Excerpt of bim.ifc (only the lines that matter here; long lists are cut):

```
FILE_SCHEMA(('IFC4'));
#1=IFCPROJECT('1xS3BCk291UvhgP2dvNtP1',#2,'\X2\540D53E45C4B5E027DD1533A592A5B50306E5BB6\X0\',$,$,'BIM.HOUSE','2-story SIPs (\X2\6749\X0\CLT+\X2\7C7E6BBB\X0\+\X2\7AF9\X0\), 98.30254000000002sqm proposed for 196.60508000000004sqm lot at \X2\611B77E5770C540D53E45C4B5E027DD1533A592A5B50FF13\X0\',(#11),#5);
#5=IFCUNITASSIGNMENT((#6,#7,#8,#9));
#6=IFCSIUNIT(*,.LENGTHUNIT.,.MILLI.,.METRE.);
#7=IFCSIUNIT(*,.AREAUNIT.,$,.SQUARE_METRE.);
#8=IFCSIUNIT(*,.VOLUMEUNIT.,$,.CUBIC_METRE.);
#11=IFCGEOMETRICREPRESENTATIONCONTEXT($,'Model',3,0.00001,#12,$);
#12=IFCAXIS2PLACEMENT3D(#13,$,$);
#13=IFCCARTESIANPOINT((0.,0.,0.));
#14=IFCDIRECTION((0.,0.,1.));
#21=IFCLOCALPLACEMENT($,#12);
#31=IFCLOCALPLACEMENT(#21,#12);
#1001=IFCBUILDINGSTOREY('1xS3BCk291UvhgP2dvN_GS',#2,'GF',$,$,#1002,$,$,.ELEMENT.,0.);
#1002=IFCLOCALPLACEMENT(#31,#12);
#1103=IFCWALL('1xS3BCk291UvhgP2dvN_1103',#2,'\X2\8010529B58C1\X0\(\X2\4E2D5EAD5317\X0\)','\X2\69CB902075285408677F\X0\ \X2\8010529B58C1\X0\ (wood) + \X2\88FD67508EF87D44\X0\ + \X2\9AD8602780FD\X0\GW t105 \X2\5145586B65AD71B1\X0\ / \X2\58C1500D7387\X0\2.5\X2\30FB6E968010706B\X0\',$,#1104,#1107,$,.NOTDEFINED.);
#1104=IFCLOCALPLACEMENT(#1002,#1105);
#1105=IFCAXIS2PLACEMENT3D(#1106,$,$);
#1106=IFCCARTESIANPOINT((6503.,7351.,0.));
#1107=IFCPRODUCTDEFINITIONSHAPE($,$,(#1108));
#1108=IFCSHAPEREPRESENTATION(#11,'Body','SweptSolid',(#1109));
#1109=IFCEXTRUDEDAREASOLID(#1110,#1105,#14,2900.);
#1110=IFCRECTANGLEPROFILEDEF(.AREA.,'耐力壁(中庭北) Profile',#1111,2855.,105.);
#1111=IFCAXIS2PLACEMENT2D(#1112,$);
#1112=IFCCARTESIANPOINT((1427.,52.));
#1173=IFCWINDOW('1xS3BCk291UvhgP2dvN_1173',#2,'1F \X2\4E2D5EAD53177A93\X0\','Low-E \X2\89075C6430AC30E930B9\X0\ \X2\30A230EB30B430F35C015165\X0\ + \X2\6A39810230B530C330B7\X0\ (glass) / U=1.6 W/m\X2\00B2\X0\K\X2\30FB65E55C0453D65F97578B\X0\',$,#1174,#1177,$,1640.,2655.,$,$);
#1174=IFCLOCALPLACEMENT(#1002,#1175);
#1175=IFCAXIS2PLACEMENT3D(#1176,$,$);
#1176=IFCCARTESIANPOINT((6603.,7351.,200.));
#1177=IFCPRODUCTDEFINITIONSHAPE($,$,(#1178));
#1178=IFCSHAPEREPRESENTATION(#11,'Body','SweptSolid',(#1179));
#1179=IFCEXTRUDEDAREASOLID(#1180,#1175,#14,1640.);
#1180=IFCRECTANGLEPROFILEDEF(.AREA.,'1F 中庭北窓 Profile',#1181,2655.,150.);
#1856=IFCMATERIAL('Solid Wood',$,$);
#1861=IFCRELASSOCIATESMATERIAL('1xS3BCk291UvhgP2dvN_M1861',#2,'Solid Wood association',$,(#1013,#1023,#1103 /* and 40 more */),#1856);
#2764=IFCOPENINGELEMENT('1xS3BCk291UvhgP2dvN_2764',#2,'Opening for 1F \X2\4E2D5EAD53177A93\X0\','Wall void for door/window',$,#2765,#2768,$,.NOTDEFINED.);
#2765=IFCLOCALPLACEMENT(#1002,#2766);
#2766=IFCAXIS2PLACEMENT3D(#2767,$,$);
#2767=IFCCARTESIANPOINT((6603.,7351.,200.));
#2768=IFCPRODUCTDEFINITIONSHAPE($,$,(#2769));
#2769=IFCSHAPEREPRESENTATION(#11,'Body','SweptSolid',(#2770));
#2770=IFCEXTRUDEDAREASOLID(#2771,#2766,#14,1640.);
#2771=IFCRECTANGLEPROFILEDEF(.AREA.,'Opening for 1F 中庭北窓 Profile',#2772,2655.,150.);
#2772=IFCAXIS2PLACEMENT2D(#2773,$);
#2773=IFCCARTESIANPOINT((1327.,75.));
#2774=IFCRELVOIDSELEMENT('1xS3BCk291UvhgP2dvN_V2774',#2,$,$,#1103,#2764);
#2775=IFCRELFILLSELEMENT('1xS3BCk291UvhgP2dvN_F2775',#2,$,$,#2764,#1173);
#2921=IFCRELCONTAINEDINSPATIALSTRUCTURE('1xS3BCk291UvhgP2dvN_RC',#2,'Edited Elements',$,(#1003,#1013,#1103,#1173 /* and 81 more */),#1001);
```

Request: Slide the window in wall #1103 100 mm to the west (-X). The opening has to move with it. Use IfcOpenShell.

```python
import ifcopenshell
import ifcopenshell.api.geometry
import ifcopenshell.util.placement
import ifcopenshell.util.unit

model = ifcopenshell.open("bim.ifc")
unit_scale = ifcopenshell.util.unit.calculate_unit_scale(model)

window = model.by_id(1173)
opening = window.FillsVoids[0].RelatingOpeningElement
wall = opening.VoidsElements[0].RelatingBuildingElement

wall_matrix = ifcopenshell.util.placement.get_local_placement(wall.ObjectPlacement)
shift = wall_matrix[:3, 0] * -0.1 / unit_scale
before = ifcopenshell.util.placement.get_local_placement(window.ObjectPlacement)[:3, 3].copy()

# The window is not placed relative to its opening, so move both.
for product in (opening, window):
    matrix = ifcopenshell.util.placement.get_local_placement(product.ObjectPlacement)
    matrix[:3, 3] += shift
    ifcopenshell.api.geometry.edit_object_placement(model, product=product, matrix=matrix, is_si=False)

after = ifcopenshell.util.placement.get_local_placement(window.ObjectPlacement)[:3, 3]
print("window moved by", (after - before).round(3) + 0.0)

model.write("bim_updated.ifc")
```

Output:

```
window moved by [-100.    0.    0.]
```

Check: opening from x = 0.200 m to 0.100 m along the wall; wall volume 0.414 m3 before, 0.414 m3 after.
